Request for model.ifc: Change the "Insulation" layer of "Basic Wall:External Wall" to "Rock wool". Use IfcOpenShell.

First a look at what the model holds.

```python
import ifcopenshell
import ifcopenshell.util.element

model = ifcopenshell.open("model.ifc")
print(model.schema)
for layer_set in model.by_type("IfcMaterialLayerSet"):
    if layer_set.LayerSetName == "Basic Wall:External Wall":
        for layer in layer_set.MaterialLayers:
            print(layer.id(), layer.Material and layer.Material.Name, layer.LayerThickness, sep=" | ")
        print(len(ifcopenshell.util.element.get_elements_by_material(model, layer_set)), "elements and types use it")
print(sorted(m.Name for m in model.by_type("IfcMaterial") if m.Name)[:60])
```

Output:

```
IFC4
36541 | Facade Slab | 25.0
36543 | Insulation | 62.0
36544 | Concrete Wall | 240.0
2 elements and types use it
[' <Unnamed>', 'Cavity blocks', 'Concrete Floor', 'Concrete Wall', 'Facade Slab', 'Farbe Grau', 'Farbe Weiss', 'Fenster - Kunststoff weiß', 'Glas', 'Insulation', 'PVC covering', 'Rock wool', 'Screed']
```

```python
import ifcopenshell
import ifcopenshell.api.material

model = ifcopenshell.open("model.ifc")

layer_set = next(s for s in model.by_type("IfcMaterialLayerSet") if s.LayerSetName == "Basic Wall:External Wall")
layer = next(l for l in layer_set.MaterialLayers if l.Material and l.Material.Name == "Insulation")
material = next(m for m in model.by_type("IfcMaterial") if m.Name == "Rock wool")

# Point this one layer at the other material; renaming the old one would change it everywhere.
ifcopenshell.api.material.edit_layer(model, layer=layer, attributes={}, material=material)

print([l.Material.Name if l.Material else None for l in layer_set.MaterialLayers])

model.write("model_rev.ifc")
```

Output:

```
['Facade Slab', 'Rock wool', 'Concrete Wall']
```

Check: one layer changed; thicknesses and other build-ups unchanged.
